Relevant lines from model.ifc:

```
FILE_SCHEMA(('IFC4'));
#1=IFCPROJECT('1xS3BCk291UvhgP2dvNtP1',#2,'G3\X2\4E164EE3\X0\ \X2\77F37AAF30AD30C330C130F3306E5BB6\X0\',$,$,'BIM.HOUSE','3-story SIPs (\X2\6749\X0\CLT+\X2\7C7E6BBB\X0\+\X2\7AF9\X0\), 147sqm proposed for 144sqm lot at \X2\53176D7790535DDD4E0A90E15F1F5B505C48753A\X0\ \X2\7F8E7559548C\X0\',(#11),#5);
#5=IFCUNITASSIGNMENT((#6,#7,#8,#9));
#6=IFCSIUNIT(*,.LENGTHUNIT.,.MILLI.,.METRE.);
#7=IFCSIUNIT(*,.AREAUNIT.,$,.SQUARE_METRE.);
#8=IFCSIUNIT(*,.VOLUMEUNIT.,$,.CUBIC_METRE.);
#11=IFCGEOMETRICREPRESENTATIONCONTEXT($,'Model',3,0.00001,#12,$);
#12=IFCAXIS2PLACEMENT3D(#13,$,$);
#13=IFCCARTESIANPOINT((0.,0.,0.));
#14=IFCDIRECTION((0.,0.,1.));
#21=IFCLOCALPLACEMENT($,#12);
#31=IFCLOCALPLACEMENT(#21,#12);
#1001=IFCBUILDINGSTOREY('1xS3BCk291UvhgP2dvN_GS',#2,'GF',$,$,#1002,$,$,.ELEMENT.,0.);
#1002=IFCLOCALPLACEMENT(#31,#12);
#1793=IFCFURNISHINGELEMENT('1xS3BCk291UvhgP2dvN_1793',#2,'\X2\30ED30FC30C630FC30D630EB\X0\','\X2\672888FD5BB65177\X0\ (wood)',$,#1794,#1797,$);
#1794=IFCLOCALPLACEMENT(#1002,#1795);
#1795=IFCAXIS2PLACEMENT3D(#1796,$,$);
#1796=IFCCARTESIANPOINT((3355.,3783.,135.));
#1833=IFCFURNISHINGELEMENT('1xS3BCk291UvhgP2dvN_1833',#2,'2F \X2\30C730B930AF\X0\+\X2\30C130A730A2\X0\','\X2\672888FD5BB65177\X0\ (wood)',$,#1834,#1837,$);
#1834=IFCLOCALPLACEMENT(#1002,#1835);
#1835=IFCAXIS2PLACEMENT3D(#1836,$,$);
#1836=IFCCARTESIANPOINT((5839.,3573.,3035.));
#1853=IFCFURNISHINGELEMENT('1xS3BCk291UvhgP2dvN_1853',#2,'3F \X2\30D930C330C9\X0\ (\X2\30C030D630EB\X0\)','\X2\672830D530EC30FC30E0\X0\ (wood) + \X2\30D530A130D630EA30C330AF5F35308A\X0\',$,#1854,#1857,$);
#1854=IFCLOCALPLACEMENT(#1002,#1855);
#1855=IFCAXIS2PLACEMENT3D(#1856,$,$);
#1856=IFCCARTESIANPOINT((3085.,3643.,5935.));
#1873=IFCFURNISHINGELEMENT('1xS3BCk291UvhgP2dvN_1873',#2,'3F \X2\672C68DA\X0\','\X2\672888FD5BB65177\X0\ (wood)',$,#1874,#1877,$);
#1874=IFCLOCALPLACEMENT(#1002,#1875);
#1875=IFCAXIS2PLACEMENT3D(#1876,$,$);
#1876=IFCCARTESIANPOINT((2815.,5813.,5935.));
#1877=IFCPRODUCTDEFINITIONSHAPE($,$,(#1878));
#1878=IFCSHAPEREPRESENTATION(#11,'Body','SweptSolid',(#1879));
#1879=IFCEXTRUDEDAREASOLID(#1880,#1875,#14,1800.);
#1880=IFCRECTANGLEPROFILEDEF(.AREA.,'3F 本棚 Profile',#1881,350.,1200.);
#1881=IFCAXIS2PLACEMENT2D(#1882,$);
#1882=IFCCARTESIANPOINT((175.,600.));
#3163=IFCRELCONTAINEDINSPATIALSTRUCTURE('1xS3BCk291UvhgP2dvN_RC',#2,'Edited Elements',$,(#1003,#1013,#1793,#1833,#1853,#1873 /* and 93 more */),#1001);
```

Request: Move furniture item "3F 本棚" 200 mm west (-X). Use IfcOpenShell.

```python
import ifcopenshell
import ifcopenshell.api.geometry
import ifcopenshell.util.placement

model = ifcopenshell.open("model.ifc")

item = model.by_id(1873)
matrix = ifcopenshell.util.placement.get_local_placement(item.ObjectPlacement)
matrix[0, 3] -= 200.0
ifcopenshell.api.geometry.edit_object_placement(model, product=item, matrix=matrix, is_si=False)

print(ifcopenshell.util.placement.get_local_placement(item.ObjectPlacement).round(3) + 0.0)

model.write("model_updated.ifc")
```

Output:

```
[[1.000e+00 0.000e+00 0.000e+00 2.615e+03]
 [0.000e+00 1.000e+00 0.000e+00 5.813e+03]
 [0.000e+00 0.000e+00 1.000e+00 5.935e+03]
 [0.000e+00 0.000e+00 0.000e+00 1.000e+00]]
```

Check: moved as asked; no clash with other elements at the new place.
